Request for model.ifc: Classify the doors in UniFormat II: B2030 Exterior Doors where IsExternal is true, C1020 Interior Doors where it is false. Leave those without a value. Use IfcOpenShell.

First a look at what the model holds.

```python
import ifcopenshell
import ifcopenshell.util.element

model = ifcopenshell.open("model.ifc")
print(model.schema)
print("classifications:", [c.Name for c in model.by_type("IfcClassification")])
values = [ifcopenshell.util.element.get_pset(e, "Pset_DoorCommon", "IsExternal") for e in model.by_type("IfcDoor")]
for value in (True, False, None):
    print("IsExternal", value, values.count(value))
```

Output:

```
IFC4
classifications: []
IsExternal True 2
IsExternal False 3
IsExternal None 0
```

```python
import ifcopenshell
import ifcopenshell.api.classification
import ifcopenshell.util.element

model = ifcopenshell.open("model.ifc")

system = ifcopenshell.api.classification.add_classification(model, classification="UniFormat II")

doors = model.by_type("IfcDoor")
external = {e: ifcopenshell.util.element.get_pset(e, "Pset_DoorCommon", "IsExternal") for e in doors}
for flag, code, name in ((True, "B2030", "Exterior Doors"), (False, "C1020", "Interior Doors")):
    products = [e for e in doors if external[e] is flag]
    ifcopenshell.api.classification.add_reference(
        model, products=products, classification=system, identification=code, name=name
    )
    print(code, len(products))

model.write("model-out.ifc")
```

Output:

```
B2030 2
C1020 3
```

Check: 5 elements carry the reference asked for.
